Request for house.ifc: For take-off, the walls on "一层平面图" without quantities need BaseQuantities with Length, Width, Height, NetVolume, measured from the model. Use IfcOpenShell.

First a look at what the model holds.

```python
import ifcopenshell
import ifcopenshell.util.element
import ifcopenshell.util.unit

model = ifcopenshell.open("house.ifc")
print(model.schema)
for unit_type in ("LENGTHUNIT", "AREAUNIT", "VOLUMEUNIT"):
    print(unit_type, ifcopenshell.util.unit.calculate_unit_scale(model, unit_type))
storey = next(s for s in model.by_type("IfcBuildingStorey") if s.Name == "一层平面图")
walls = [e for e in ifcopenshell.util.element.get_decomposition(storey) if e.is_a("IfcWall")]
for e in sorted(walls, key=lambda e: e.id()):
    print(e.id(), e.is_a(), e.Name, list(ifcopenshell.util.element.get_psets(e, qtos_only=True)), sep=" | ")
```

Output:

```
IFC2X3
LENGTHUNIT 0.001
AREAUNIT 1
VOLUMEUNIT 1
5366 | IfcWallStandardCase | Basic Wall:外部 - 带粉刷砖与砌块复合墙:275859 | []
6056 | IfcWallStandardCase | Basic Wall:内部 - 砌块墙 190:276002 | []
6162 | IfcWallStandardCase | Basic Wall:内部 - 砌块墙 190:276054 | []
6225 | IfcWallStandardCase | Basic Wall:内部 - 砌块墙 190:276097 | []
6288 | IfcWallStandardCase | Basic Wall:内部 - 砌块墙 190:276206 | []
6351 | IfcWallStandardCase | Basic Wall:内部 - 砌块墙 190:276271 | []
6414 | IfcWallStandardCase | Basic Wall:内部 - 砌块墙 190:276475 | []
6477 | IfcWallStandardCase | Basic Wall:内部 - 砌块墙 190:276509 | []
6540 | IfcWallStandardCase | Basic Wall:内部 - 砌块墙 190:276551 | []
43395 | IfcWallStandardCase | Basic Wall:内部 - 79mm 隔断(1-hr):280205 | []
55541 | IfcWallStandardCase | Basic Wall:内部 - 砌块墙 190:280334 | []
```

```python
import ifcopenshell
import ifcopenshell.api.pset
import ifcopenshell.geom
import ifcopenshell.util.element
import ifcopenshell.util.shape
import ifcopenshell.util.unit

model = ifcopenshell.open("house.ifc")
unit_scale = ifcopenshell.util.unit.calculate_unit_scale(model)
volume_scale = ifcopenshell.util.unit.calculate_unit_scale(model, "VOLUMEUNIT")
settings = ifcopenshell.geom.settings()

storey = next(s for s in model.by_type("IfcBuildingStorey") if s.Name == "一层平面图")
walls = [e for e in ifcopenshell.util.element.get_decomposition(storey) if e.is_a("IfcWall")]

for e in sorted(walls, key=lambda e: e.id()):
    if ifcopenshell.util.element.get_psets(e, qtos_only=True, should_inherit=False):
        continue
    # Geometry comes back in metres, in the element's own axes.
    shape = ifcopenshell.geom.create_shape(settings, e)
    values = {
        "Length": ifcopenshell.util.shape.get_x(shape.geometry) / unit_scale,
        "Width": ifcopenshell.util.shape.get_y(shape.geometry) / unit_scale,
        "Height": ifcopenshell.util.shape.get_z(shape.geometry) / unit_scale,
        "NetVolume": ifcopenshell.util.shape.get_volume(shape.geometry) / volume_scale,
    }
    qto = ifcopenshell.api.pset.add_qto(model, product=e, name="BaseQuantities")
    ifcopenshell.api.pset.edit_qto(model, qto=qto, properties=values)
    print(e.id(), {k: round(v, 3) for k, v in values.items()})

model.write("house-out.ifc")
```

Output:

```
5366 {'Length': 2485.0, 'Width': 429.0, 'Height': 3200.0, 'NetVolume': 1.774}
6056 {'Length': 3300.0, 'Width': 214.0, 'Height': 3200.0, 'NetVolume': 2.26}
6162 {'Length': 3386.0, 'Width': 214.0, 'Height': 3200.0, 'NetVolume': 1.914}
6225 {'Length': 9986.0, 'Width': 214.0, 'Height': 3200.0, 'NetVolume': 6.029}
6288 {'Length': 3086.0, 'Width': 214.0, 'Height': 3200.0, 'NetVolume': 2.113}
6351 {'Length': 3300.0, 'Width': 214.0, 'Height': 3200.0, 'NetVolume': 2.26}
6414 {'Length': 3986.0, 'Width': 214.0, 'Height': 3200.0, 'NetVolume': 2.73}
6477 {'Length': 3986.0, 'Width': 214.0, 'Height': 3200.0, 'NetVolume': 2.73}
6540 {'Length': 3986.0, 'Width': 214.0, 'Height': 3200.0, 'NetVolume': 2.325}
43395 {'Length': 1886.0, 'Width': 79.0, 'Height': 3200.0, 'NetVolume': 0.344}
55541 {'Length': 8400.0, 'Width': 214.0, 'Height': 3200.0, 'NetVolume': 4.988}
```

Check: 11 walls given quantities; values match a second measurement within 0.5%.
